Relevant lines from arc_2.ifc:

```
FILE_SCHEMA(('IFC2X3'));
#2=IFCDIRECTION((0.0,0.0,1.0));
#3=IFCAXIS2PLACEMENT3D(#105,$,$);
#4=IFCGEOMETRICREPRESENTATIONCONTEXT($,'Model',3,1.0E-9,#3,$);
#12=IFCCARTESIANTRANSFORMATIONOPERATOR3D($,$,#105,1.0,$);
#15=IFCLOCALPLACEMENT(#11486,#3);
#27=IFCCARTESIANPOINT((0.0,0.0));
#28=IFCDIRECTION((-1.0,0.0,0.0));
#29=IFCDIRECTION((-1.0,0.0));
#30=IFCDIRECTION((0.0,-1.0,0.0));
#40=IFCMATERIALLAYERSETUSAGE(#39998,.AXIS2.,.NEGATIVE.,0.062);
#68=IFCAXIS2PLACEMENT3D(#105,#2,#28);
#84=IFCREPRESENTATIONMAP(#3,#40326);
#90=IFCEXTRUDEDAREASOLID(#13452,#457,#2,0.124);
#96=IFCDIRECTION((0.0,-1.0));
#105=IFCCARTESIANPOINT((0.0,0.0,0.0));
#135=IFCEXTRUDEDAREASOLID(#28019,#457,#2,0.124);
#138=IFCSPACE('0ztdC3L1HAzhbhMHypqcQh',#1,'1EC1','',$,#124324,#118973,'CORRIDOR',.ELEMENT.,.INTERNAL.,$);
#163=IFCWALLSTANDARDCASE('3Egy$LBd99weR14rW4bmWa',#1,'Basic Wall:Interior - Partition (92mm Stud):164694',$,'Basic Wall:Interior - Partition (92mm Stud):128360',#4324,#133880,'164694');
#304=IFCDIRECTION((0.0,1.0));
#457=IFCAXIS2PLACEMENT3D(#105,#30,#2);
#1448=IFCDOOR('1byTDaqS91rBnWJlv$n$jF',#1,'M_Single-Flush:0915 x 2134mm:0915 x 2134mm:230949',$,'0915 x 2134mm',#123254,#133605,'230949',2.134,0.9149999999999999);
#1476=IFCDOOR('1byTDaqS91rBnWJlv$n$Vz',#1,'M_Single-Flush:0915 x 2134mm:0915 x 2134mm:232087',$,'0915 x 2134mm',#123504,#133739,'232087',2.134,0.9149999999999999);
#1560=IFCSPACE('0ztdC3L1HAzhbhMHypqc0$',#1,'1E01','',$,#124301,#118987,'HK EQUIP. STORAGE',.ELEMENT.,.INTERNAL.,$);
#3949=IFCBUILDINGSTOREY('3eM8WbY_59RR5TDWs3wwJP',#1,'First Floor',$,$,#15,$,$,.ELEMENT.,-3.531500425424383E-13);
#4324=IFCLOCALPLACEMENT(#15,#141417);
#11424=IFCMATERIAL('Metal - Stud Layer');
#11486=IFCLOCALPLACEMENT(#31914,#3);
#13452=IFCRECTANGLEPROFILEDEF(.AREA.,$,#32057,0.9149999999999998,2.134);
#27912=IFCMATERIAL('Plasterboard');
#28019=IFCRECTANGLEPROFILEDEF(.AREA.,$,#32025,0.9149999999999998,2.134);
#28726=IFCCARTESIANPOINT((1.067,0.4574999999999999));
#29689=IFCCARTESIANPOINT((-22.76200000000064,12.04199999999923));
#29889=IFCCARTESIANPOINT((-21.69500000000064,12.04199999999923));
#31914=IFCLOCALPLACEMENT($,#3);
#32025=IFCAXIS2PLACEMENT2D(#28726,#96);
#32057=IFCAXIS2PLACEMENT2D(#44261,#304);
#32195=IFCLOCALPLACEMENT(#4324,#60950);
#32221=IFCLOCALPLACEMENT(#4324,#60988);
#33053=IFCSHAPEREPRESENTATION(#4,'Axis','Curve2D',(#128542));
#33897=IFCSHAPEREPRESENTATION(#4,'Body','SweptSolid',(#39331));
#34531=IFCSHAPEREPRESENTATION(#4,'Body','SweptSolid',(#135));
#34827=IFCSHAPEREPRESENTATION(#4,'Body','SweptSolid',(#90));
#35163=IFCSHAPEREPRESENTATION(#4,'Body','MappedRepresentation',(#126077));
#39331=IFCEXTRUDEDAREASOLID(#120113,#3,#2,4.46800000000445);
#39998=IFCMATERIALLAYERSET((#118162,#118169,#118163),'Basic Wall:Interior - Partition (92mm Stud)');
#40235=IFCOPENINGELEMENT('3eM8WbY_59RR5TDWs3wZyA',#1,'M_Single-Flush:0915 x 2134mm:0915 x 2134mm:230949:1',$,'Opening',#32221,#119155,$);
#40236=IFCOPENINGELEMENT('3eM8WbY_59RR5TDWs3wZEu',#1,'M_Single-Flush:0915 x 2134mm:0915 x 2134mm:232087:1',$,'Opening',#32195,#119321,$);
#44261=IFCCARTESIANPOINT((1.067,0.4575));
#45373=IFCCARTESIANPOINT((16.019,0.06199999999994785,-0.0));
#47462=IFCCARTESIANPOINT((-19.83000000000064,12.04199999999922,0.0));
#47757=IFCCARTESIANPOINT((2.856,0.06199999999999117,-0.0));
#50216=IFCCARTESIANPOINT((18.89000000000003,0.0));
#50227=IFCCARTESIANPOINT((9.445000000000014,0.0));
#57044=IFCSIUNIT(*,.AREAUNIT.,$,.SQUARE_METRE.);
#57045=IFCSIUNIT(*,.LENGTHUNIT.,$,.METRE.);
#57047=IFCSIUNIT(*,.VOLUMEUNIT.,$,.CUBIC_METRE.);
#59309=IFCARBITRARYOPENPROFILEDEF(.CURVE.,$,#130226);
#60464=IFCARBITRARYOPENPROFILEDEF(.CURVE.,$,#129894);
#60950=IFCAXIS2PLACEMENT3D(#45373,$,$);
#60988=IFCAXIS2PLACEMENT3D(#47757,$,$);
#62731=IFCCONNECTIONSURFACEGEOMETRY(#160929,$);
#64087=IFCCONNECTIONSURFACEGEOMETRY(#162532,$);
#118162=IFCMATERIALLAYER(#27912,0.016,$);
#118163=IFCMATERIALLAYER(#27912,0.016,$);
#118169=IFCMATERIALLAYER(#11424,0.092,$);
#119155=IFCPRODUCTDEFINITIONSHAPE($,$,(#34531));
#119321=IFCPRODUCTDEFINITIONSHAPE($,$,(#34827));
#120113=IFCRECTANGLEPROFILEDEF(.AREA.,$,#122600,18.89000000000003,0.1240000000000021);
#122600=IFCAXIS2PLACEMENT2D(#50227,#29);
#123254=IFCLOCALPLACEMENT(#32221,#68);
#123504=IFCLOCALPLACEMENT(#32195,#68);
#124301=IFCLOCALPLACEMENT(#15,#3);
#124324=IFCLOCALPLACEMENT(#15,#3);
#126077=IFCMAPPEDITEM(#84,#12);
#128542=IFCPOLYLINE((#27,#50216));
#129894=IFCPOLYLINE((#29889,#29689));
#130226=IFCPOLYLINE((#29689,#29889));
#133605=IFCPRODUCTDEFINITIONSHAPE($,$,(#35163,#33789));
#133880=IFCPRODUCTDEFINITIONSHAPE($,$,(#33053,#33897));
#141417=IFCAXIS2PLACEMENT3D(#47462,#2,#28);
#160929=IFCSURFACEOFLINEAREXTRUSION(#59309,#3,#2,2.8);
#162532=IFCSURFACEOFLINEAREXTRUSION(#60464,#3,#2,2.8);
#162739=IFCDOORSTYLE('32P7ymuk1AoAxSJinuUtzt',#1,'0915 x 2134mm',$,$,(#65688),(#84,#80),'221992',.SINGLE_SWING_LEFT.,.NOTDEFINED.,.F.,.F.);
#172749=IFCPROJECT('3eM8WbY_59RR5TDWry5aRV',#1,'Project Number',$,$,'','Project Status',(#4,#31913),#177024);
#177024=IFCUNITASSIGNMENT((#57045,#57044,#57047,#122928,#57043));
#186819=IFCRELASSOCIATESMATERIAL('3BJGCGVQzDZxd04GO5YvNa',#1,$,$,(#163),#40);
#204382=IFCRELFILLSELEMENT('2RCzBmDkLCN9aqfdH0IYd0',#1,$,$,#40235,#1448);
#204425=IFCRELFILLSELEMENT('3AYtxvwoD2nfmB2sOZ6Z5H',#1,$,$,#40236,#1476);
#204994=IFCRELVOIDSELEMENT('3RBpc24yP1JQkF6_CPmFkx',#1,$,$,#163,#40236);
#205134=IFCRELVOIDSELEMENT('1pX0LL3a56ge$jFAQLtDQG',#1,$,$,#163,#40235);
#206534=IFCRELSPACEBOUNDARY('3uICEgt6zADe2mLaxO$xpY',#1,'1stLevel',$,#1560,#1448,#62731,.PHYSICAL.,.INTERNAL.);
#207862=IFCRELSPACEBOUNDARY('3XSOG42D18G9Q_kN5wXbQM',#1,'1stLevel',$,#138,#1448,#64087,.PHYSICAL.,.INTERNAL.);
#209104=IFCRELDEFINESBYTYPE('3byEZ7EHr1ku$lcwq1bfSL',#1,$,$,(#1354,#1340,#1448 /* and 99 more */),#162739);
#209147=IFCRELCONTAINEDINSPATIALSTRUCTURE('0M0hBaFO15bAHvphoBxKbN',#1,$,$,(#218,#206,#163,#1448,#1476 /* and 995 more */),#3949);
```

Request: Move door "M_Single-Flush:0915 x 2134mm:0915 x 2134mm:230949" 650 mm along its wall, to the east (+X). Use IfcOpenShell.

```python
import numpy as np
import ifcopenshell
import ifcopenshell.api.geometry
import ifcopenshell.util.placement
import ifcopenshell.util.unit

model = ifcopenshell.open("arc_2.ifc")
unit_scale = ifcopenshell.util.unit.calculate_unit_scale(model)

door = model.by_id(1448)
opening = door.FillsVoids[0].RelatingOpeningElement
wall = opening.VoidsElements[0].RelatingBuildingElement

wall_matrix = ifcopenshell.util.placement.get_local_placement(wall.ObjectPlacement)
shift = wall_matrix[:3, 0] * -0.65 / unit_scale
before = ifcopenshell.util.placement.get_local_placement(door.ObjectPlacement)[:3, 3].copy()

# The door is placed relative to its opening, so it follows when the opening moves.
matrix = ifcopenshell.util.placement.get_local_placement(opening.ObjectPlacement)
matrix[:3, 3] += shift
ifcopenshell.api.geometry.edit_object_placement(
    model, product=opening, matrix=matrix, is_si=False, should_transform_children=True
)

# Space boundary surfaces are stored in each space's coordinates; move them too.
for rel in door.ProvidesBoundaries:
    if not rel.ConnectionGeometry:
        continue
    surface = rel.ConnectionGeometry.SurfaceOnRelatingElement
    space_matrix = ifcopenshell.util.placement.get_local_placement(rel.RelatingSpace.ObjectPlacement)
    point = np.array(surface.Position.Location.Coordinates) + space_matrix[:3, :3].T @ shift
    surface.Position = model.createIfcAxis2Placement3D(
        model.createIfcCartesianPoint(point.tolist()), surface.Position.Axis, surface.Position.RefDirection
    )

after = ifcopenshell.util.placement.get_local_placement(door.ObjectPlacement)[:3, 3]
print("door moved by", (after - before).round(3) + 0.0)

model.write("arc_2_updated.ifc")
```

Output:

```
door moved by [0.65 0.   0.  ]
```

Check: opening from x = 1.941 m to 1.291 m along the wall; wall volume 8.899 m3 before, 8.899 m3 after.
